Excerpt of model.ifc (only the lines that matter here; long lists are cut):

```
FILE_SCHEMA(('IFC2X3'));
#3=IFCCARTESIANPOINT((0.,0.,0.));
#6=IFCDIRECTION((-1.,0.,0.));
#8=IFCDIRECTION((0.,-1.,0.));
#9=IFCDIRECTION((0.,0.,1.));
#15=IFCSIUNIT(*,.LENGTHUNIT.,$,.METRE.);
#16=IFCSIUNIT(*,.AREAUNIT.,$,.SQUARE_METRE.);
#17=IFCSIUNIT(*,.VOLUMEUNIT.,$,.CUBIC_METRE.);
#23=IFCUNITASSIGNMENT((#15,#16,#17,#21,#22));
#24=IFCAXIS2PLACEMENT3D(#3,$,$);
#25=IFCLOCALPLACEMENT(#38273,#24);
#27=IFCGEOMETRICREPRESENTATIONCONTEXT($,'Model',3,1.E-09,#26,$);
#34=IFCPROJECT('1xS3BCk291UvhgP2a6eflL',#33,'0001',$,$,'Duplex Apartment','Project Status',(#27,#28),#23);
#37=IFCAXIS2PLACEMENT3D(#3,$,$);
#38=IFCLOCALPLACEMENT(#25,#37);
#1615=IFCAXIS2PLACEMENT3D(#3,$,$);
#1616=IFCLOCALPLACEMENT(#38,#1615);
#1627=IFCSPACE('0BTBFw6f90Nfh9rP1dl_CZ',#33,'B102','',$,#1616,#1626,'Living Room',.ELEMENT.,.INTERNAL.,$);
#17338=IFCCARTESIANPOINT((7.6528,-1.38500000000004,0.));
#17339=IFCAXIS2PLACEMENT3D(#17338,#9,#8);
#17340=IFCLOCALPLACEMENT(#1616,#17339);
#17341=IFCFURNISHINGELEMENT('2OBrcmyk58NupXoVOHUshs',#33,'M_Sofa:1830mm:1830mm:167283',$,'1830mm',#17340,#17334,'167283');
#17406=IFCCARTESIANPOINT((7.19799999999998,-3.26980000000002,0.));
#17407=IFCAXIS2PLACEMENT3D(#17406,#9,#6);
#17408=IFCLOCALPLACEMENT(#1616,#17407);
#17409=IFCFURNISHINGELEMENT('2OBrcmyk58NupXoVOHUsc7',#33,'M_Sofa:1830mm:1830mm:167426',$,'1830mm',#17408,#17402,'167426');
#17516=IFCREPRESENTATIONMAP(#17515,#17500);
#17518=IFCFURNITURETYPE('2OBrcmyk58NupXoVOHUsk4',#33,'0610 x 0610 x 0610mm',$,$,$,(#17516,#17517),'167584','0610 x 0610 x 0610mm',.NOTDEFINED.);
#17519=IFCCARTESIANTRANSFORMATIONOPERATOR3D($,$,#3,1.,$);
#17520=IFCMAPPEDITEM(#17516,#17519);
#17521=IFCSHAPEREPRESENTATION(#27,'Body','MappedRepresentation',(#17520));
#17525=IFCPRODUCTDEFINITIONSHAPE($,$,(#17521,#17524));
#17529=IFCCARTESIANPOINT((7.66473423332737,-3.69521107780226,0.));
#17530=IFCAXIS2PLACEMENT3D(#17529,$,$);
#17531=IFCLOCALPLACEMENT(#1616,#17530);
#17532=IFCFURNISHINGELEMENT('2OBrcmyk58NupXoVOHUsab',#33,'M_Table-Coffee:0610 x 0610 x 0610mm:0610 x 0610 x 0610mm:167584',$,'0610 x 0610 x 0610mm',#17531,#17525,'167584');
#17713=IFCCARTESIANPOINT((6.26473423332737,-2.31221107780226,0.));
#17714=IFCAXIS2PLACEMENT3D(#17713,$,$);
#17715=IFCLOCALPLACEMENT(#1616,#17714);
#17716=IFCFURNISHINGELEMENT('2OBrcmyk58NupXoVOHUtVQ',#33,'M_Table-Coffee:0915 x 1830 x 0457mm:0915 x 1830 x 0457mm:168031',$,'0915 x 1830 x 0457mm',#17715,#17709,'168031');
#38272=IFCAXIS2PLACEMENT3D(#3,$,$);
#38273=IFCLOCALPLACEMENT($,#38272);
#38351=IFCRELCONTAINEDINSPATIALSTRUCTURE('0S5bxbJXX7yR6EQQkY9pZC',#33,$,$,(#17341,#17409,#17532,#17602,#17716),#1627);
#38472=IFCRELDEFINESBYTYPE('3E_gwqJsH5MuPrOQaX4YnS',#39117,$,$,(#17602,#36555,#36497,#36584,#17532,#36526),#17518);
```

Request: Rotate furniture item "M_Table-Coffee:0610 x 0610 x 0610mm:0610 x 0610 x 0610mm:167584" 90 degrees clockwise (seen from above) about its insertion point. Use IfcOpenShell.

```python
import ifcopenshell
import ifcopenshell.api.geometry
import ifcopenshell.util.placement

model = ifcopenshell.open("model.ifc")

item = model.by_guid("2OBrcmyk58NupXoVOHUsab")
matrix = ifcopenshell.util.placement.get_local_placement(item.ObjectPlacement)
matrix = matrix @ ifcopenshell.util.placement.rotation(-90, "Z")
ifcopenshell.api.geometry.edit_object_placement(model, product=item, matrix=matrix, is_si=False)

print(ifcopenshell.util.placement.get_local_placement(item.ObjectPlacement).round(3) + 0.0)

model.write("model-out.ifc")
```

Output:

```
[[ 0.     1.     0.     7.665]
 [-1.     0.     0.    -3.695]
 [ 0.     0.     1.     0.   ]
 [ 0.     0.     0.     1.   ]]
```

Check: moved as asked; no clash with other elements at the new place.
